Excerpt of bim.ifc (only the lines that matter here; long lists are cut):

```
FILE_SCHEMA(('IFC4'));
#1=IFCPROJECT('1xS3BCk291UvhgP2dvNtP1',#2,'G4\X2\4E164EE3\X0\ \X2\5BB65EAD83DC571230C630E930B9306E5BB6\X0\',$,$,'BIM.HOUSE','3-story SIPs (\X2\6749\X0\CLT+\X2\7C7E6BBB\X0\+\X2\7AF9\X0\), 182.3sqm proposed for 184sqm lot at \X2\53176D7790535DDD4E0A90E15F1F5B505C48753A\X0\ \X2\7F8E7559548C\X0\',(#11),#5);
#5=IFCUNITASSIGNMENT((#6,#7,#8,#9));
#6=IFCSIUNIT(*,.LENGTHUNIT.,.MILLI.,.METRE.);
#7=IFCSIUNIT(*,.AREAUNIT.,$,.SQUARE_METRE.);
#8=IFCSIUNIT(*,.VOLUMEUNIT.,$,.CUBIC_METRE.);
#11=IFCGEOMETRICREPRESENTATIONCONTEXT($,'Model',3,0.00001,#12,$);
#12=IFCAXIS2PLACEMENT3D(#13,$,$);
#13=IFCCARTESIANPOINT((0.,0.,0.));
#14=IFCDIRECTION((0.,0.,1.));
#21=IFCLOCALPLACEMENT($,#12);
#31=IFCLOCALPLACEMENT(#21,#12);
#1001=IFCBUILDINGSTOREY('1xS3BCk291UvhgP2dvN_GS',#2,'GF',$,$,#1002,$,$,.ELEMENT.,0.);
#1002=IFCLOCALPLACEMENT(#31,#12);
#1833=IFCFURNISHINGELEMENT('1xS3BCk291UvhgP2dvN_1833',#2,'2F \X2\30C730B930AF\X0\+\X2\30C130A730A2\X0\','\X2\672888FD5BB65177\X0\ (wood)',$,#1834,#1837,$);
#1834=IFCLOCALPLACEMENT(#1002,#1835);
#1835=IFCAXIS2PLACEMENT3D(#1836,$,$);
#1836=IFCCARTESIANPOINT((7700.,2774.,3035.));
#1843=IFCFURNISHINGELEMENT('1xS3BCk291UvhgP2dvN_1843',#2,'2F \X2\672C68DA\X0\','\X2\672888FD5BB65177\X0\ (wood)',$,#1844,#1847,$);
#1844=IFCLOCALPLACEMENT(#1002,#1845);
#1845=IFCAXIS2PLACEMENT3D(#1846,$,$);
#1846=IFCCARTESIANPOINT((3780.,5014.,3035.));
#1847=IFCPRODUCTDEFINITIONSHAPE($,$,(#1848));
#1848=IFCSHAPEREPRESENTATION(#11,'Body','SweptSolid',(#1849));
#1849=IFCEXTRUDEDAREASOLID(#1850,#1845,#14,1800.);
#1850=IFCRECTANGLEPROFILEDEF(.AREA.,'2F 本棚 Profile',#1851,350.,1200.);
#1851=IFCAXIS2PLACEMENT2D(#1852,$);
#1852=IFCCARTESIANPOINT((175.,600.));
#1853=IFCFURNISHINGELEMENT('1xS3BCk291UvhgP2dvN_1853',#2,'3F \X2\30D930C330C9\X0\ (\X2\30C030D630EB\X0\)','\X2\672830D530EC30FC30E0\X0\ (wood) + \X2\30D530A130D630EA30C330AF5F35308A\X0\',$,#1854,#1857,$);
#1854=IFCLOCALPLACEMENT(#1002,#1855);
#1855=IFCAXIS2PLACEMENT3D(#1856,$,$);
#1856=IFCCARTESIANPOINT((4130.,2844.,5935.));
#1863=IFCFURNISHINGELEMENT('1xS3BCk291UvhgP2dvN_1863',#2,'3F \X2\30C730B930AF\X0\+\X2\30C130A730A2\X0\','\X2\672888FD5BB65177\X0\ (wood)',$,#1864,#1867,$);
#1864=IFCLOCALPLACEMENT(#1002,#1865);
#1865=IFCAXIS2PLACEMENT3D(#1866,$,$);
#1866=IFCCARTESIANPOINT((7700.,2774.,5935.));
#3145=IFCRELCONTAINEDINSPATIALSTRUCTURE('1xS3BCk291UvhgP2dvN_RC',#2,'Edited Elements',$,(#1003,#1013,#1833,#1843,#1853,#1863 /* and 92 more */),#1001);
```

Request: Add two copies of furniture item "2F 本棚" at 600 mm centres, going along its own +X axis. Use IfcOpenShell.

```python
import ifcopenshell
import ifcopenshell.api.geometry
import ifcopenshell.api.root
import ifcopenshell.util.element
import ifcopenshell.util.placement
import ifcopenshell.util.unit

model = ifcopenshell.open("bim.ifc")
unit_scale = ifcopenshell.util.unit.calculate_unit_scale(model)


def reuse_history(source, copy):
    """copy_class also copies each property set's owner history, people and application; keep the originals."""
    for rel in copy.IsDefinedBy:
        if rel.is_a("IfcRelDefinesByProperties") and (history := rel.RelatingPropertyDefinition.OwnerHistory):
            rel.RelatingPropertyDefinition.OwnerHistory = source.OwnerHistory
            ifcopenshell.util.element.remove_deep2(model, history)


source = model.by_id(1843)
base = ifcopenshell.util.placement.get_local_placement(source.ObjectPlacement)
step = base[:3, 0] * 0.6 / unit_scale

for i in range(1, 3):
    copy = ifcopenshell.api.root.copy_class(model, product=source)
    copy.Representation = ifcopenshell.util.element.copy_deep(
        model, source.Representation, exclude=["IfcGeometricRepresentationContext", "IfcRepresentationMap"]
    )
    reuse_history(source, copy)
    matrix = base.copy()
    matrix[:3, 3] += i * step
    print("added at", matrix[:3, 3].round(3) + 0.0)
    ifcopenshell.api.geometry.edit_object_placement(model, product=copy, matrix=matrix, is_si=False)

model.write("bim_edited.ifc")
```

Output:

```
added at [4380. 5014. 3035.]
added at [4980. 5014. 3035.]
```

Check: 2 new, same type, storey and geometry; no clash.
